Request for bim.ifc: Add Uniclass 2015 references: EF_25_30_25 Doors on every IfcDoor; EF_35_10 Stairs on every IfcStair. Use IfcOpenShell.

First a look at what the model holds.

```python
import ifcopenshell

model = ifcopenshell.open("bim.ifc")
print(model.schema)
print("classifications:", [c.Name for c in model.by_type("IfcClassification")])
for ifc_class in ("IfcDoor", "IfcRoof", "IfcStair", "IfcWall", "IfcWindow"):
    print(ifc_class, len(model.by_type(ifc_class)))
```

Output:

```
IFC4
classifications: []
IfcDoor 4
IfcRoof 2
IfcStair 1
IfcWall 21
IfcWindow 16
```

```python
import ifcopenshell
import ifcopenshell.api.classification

model = ifcopenshell.open("bim.ifc")

system = ifcopenshell.api.classification.add_classification(model, classification="Uniclass 2015")

codes = {
    "IfcDoor": ("EF_25_30_25", "Doors"),
    "IfcStair": ("EF_35_10", "Stairs"),
}
for ifc_class, (code, name) in codes.items():
    products = model.by_type(ifc_class)
    ifcopenshell.api.classification.add_reference(
        model, products=products, classification=system, identification=code, name=name
    )
    print(code, len(products))

model.write("bim-out.ifc")
```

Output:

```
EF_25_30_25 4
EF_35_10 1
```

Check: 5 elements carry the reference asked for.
